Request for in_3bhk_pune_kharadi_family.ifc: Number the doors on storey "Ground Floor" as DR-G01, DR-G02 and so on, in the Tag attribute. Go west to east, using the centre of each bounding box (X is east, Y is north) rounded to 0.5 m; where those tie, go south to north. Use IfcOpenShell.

First a look at what the model holds.

```python
import ifcopenshell
import ifcopenshell.util.element
import ifcopenshell.util.placement

model = ifcopenshell.open("in_3bhk_pune_kharadi_family.ifc")
print(model.schema)
storey = next(s for s in model.by_type("IfcBuildingStorey") if s.Name == "Ground Floor")
doors = [e for e in ifcopenshell.util.element.get_decomposition(storey) if e.is_a("IfcDoor")]
for e in sorted(doors, key=lambda e: e.id()):
    origin = ifcopenshell.util.placement.get_local_placement(e.ObjectPlacement)[:3, 3]
    print(e.id(), e.Tag, e.Name, origin.round(2) + 0.0, sep=" | ")
```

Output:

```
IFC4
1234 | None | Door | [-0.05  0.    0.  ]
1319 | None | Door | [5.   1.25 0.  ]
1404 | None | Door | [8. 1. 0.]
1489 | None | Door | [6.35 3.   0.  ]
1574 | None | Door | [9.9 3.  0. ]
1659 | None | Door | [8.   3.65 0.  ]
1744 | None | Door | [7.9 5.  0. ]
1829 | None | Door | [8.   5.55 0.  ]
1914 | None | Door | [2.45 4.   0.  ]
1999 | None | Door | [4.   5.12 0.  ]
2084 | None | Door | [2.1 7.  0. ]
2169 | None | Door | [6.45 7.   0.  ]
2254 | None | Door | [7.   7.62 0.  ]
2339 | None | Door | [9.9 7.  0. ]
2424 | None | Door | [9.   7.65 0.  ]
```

```python
import ifcopenshell
import ifcopenshell.geom
import ifcopenshell.util.element
import ifcopenshell.util.shape

model = ifcopenshell.open("in_3bhk_pune_kharadi_family.ifc")
settings = ifcopenshell.geom.settings()
settings.set("use-world-coords", True)


def centre(element):
    shape = ifcopenshell.geom.create_shape(settings, element)
    return ifcopenshell.util.shape.get_bbox_centroid(shape.geometry)


storey = next(s for s in model.by_type("IfcBuildingStorey") if s.Name == "Ground Floor")
doors = [e for e in ifcopenshell.util.element.get_decomposition(storey) if e.is_a("IfcDoor")]

# Insertion points can sit at a corner or the storey origin, so sort by the geometry (in metres).
centres = {e: centre(e) for e in doors}
doors.sort(key=lambda e: (round(centres[e][0] / 0.5), centres[e][1]))

for i, e in enumerate(doors, start=1):
    number = f"DR-G{i:02d}"
    e.Tag = number
    print(e.id(), number)

model.write("in_3bhk_pune_kharadi_family_updated.ifc")
```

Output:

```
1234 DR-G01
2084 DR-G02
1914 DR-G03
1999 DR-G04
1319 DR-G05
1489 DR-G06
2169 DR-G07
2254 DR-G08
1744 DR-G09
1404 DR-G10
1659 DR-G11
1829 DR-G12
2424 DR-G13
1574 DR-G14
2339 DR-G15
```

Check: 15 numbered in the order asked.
